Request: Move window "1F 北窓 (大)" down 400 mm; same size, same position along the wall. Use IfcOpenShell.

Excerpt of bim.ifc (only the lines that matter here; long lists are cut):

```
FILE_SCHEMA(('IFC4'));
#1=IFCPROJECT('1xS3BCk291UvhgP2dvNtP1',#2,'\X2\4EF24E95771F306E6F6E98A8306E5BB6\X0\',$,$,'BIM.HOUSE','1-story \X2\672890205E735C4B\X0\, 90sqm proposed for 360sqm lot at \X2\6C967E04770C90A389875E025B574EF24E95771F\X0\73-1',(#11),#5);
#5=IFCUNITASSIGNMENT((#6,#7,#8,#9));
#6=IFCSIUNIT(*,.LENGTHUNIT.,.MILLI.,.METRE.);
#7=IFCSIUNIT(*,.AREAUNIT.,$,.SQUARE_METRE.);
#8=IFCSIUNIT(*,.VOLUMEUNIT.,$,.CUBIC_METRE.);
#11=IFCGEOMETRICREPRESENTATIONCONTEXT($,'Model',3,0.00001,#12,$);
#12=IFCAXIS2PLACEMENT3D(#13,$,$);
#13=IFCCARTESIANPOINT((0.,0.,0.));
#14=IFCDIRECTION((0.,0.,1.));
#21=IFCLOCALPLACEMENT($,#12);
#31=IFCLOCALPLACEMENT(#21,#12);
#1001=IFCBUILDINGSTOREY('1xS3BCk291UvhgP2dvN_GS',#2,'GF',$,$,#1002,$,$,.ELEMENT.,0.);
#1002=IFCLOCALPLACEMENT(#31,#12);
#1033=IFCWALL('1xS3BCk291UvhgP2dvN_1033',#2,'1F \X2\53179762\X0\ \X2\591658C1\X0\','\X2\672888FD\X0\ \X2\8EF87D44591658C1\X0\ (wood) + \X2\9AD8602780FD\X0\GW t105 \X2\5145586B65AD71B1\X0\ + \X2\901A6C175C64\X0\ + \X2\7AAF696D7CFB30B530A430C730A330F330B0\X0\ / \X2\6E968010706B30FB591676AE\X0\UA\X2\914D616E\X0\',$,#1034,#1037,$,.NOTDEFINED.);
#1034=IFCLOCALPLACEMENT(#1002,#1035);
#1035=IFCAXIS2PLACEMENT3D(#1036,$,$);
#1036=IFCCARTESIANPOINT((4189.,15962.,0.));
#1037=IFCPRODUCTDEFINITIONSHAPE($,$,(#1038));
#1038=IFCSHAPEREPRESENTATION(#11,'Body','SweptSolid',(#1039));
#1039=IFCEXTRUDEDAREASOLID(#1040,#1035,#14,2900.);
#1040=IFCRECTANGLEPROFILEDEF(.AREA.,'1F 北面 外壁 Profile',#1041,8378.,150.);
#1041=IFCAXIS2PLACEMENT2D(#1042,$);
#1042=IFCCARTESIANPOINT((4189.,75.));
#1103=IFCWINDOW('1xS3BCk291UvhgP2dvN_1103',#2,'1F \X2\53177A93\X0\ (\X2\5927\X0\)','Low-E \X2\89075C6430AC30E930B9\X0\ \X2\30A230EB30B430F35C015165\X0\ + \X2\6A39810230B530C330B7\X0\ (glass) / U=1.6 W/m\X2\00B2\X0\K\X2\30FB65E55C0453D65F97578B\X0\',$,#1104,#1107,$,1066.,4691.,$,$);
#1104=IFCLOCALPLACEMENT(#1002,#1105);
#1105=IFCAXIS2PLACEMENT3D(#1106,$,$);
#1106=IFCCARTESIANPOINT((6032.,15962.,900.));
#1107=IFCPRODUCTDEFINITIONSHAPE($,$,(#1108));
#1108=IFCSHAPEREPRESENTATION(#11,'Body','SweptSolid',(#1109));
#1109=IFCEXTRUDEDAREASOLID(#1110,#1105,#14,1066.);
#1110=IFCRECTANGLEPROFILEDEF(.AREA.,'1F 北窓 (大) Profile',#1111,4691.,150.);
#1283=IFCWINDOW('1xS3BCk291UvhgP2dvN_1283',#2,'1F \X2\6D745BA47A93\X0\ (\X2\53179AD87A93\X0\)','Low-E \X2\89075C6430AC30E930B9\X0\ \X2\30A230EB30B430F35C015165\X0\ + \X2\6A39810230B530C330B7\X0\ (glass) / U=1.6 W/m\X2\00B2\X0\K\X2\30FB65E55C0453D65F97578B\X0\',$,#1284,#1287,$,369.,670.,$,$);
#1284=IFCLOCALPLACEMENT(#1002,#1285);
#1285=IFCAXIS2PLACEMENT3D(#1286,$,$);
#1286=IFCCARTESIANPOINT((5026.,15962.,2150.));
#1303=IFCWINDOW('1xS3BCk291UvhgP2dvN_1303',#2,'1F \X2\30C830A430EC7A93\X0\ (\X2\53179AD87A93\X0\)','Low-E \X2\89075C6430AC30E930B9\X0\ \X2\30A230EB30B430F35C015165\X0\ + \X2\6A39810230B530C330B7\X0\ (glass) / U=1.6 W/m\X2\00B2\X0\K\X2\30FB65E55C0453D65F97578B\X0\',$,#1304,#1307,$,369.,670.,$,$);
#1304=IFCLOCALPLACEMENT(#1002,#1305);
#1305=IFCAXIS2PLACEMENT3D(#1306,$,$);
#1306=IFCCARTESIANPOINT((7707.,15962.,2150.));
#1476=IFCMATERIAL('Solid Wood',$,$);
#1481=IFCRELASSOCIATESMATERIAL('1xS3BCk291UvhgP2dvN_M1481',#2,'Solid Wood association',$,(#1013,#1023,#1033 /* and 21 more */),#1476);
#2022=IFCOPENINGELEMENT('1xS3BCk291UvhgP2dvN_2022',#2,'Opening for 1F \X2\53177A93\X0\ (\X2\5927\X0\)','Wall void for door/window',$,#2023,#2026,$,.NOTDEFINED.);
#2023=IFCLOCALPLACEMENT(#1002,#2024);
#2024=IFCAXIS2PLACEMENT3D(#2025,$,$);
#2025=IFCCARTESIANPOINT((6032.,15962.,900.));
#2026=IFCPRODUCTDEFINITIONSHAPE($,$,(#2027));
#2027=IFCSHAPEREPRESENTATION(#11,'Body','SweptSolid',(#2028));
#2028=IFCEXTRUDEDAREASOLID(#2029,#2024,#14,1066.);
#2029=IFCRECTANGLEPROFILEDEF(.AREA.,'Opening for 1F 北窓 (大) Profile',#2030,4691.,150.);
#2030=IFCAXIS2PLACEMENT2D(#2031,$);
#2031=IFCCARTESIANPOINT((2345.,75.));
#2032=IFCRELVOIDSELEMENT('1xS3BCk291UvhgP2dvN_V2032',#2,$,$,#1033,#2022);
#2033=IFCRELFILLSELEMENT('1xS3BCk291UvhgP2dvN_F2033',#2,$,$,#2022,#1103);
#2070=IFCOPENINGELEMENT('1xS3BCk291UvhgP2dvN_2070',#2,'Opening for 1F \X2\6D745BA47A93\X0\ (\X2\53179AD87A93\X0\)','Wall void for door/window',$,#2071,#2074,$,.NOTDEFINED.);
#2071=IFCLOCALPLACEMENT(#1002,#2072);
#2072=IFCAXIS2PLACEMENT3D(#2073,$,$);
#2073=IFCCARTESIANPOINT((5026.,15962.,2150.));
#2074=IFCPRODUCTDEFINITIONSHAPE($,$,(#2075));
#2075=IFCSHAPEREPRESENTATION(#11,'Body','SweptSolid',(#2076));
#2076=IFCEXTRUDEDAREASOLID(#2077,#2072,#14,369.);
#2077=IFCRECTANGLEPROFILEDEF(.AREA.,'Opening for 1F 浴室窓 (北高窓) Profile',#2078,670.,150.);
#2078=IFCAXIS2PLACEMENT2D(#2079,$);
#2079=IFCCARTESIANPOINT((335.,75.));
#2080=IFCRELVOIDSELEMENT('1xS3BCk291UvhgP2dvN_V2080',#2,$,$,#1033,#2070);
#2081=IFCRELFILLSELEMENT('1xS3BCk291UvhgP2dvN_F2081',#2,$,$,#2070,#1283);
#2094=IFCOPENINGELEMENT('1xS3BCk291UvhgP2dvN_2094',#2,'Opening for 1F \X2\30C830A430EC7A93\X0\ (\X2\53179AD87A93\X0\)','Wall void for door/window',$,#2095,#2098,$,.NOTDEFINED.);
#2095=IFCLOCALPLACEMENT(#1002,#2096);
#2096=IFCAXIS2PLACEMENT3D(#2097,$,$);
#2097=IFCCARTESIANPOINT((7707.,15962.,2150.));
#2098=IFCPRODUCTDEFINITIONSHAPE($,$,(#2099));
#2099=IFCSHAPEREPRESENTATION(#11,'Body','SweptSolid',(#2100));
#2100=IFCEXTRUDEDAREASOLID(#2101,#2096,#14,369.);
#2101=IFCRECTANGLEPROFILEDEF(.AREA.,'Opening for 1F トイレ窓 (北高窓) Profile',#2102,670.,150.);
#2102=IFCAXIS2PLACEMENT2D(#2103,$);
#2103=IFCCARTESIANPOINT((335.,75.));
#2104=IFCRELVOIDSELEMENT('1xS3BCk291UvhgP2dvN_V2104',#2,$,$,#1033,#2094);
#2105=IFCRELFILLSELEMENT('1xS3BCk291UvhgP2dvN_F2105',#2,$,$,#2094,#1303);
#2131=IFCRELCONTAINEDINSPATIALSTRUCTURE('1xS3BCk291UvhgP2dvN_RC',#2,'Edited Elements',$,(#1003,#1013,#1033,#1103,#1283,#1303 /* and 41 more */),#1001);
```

```python
import numpy as np
import ifcopenshell
import ifcopenshell.api.geometry
import ifcopenshell.util.placement
import ifcopenshell.util.unit

model = ifcopenshell.open("bim.ifc")
unit_scale = ifcopenshell.util.unit.calculate_unit_scale(model)

window = model.by_guid("1xS3BCk291UvhgP2dvN_1103")
opening = window.FillsVoids[0].RelatingOpeningElement
dz = -0.4 / unit_scale

shift = np.array([0.0, 0.0, dz])
# The window is not placed relative to its opening, so move both.
for product in (opening, window):
    matrix = ifcopenshell.util.placement.get_local_placement(product.ObjectPlacement)
    matrix[:3, 3] += shift
    ifcopenshell.api.geometry.edit_object_placement(model, product=product, matrix=matrix, is_si=False)

print(f"moved by {dz * unit_scale:+.3f} m")

model.write("bim_updated.ifc")
```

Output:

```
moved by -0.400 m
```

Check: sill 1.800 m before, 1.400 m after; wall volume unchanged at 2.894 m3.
